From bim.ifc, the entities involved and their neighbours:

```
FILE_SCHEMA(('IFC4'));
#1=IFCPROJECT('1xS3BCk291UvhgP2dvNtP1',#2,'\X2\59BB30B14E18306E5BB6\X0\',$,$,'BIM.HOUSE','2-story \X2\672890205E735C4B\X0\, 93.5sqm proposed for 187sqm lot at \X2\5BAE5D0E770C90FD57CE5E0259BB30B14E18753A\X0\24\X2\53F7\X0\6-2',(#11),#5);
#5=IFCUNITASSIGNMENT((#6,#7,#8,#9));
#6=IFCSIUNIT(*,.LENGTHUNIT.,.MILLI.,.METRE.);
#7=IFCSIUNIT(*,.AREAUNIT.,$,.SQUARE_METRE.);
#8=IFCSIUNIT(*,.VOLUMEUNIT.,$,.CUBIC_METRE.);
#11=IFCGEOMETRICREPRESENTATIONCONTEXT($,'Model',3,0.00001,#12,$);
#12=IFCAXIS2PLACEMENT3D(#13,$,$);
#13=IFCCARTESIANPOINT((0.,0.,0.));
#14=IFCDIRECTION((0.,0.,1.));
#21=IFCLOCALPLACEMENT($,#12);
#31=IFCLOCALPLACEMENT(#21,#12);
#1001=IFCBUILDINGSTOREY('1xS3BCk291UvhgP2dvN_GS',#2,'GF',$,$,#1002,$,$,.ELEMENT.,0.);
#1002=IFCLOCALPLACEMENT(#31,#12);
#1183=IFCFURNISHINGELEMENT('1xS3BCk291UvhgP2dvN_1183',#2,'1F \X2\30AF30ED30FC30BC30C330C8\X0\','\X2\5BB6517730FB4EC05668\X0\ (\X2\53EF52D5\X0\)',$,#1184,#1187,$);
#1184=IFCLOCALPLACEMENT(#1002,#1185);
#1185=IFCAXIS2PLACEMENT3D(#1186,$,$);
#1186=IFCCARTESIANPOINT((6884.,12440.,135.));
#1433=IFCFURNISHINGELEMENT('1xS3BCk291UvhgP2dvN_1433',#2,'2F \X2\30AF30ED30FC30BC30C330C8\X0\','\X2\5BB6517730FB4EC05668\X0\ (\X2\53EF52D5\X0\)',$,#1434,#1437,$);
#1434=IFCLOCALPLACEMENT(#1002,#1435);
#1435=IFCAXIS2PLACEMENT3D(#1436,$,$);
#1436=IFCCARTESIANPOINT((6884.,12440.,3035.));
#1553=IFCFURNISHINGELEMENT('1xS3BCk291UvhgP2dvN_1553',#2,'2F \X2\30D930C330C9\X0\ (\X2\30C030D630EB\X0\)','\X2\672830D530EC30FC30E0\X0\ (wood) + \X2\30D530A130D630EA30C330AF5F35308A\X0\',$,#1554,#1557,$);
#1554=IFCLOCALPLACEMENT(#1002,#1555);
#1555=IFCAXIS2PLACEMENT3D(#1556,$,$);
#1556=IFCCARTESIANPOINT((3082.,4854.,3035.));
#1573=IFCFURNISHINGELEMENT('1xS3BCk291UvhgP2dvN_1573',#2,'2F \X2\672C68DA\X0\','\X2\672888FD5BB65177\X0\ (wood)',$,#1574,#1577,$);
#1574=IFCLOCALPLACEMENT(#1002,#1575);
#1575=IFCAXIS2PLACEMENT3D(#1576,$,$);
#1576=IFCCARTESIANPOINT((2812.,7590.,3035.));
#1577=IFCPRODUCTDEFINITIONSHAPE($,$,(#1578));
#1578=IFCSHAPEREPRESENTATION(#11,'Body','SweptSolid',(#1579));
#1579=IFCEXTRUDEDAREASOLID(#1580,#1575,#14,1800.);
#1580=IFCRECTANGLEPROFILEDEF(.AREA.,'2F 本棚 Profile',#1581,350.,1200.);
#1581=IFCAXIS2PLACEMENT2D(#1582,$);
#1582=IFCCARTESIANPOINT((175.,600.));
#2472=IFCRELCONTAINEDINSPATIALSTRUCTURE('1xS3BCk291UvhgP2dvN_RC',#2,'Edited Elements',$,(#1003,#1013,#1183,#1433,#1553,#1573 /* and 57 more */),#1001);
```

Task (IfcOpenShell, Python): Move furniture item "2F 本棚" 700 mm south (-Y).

```python
import ifcopenshell
import ifcopenshell.api.geometry
import ifcopenshell.util.placement

model = ifcopenshell.open("bim.ifc")

item = model.by_guid("1xS3BCk291UvhgP2dvN_1573")
matrix = ifcopenshell.util.placement.get_local_placement(item.ObjectPlacement)
matrix[1, 3] -= 700.0
ifcopenshell.api.geometry.edit_object_placement(model, product=item, matrix=matrix, is_si=False)

print(ifcopenshell.util.placement.get_local_placement(item.ObjectPlacement).round(3) + 0.0)

model.write("bim-out.ifc")
```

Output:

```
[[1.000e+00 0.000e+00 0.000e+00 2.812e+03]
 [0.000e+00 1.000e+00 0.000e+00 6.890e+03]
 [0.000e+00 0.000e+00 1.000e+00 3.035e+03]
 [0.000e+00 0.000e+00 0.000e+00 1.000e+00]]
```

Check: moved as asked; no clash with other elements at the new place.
